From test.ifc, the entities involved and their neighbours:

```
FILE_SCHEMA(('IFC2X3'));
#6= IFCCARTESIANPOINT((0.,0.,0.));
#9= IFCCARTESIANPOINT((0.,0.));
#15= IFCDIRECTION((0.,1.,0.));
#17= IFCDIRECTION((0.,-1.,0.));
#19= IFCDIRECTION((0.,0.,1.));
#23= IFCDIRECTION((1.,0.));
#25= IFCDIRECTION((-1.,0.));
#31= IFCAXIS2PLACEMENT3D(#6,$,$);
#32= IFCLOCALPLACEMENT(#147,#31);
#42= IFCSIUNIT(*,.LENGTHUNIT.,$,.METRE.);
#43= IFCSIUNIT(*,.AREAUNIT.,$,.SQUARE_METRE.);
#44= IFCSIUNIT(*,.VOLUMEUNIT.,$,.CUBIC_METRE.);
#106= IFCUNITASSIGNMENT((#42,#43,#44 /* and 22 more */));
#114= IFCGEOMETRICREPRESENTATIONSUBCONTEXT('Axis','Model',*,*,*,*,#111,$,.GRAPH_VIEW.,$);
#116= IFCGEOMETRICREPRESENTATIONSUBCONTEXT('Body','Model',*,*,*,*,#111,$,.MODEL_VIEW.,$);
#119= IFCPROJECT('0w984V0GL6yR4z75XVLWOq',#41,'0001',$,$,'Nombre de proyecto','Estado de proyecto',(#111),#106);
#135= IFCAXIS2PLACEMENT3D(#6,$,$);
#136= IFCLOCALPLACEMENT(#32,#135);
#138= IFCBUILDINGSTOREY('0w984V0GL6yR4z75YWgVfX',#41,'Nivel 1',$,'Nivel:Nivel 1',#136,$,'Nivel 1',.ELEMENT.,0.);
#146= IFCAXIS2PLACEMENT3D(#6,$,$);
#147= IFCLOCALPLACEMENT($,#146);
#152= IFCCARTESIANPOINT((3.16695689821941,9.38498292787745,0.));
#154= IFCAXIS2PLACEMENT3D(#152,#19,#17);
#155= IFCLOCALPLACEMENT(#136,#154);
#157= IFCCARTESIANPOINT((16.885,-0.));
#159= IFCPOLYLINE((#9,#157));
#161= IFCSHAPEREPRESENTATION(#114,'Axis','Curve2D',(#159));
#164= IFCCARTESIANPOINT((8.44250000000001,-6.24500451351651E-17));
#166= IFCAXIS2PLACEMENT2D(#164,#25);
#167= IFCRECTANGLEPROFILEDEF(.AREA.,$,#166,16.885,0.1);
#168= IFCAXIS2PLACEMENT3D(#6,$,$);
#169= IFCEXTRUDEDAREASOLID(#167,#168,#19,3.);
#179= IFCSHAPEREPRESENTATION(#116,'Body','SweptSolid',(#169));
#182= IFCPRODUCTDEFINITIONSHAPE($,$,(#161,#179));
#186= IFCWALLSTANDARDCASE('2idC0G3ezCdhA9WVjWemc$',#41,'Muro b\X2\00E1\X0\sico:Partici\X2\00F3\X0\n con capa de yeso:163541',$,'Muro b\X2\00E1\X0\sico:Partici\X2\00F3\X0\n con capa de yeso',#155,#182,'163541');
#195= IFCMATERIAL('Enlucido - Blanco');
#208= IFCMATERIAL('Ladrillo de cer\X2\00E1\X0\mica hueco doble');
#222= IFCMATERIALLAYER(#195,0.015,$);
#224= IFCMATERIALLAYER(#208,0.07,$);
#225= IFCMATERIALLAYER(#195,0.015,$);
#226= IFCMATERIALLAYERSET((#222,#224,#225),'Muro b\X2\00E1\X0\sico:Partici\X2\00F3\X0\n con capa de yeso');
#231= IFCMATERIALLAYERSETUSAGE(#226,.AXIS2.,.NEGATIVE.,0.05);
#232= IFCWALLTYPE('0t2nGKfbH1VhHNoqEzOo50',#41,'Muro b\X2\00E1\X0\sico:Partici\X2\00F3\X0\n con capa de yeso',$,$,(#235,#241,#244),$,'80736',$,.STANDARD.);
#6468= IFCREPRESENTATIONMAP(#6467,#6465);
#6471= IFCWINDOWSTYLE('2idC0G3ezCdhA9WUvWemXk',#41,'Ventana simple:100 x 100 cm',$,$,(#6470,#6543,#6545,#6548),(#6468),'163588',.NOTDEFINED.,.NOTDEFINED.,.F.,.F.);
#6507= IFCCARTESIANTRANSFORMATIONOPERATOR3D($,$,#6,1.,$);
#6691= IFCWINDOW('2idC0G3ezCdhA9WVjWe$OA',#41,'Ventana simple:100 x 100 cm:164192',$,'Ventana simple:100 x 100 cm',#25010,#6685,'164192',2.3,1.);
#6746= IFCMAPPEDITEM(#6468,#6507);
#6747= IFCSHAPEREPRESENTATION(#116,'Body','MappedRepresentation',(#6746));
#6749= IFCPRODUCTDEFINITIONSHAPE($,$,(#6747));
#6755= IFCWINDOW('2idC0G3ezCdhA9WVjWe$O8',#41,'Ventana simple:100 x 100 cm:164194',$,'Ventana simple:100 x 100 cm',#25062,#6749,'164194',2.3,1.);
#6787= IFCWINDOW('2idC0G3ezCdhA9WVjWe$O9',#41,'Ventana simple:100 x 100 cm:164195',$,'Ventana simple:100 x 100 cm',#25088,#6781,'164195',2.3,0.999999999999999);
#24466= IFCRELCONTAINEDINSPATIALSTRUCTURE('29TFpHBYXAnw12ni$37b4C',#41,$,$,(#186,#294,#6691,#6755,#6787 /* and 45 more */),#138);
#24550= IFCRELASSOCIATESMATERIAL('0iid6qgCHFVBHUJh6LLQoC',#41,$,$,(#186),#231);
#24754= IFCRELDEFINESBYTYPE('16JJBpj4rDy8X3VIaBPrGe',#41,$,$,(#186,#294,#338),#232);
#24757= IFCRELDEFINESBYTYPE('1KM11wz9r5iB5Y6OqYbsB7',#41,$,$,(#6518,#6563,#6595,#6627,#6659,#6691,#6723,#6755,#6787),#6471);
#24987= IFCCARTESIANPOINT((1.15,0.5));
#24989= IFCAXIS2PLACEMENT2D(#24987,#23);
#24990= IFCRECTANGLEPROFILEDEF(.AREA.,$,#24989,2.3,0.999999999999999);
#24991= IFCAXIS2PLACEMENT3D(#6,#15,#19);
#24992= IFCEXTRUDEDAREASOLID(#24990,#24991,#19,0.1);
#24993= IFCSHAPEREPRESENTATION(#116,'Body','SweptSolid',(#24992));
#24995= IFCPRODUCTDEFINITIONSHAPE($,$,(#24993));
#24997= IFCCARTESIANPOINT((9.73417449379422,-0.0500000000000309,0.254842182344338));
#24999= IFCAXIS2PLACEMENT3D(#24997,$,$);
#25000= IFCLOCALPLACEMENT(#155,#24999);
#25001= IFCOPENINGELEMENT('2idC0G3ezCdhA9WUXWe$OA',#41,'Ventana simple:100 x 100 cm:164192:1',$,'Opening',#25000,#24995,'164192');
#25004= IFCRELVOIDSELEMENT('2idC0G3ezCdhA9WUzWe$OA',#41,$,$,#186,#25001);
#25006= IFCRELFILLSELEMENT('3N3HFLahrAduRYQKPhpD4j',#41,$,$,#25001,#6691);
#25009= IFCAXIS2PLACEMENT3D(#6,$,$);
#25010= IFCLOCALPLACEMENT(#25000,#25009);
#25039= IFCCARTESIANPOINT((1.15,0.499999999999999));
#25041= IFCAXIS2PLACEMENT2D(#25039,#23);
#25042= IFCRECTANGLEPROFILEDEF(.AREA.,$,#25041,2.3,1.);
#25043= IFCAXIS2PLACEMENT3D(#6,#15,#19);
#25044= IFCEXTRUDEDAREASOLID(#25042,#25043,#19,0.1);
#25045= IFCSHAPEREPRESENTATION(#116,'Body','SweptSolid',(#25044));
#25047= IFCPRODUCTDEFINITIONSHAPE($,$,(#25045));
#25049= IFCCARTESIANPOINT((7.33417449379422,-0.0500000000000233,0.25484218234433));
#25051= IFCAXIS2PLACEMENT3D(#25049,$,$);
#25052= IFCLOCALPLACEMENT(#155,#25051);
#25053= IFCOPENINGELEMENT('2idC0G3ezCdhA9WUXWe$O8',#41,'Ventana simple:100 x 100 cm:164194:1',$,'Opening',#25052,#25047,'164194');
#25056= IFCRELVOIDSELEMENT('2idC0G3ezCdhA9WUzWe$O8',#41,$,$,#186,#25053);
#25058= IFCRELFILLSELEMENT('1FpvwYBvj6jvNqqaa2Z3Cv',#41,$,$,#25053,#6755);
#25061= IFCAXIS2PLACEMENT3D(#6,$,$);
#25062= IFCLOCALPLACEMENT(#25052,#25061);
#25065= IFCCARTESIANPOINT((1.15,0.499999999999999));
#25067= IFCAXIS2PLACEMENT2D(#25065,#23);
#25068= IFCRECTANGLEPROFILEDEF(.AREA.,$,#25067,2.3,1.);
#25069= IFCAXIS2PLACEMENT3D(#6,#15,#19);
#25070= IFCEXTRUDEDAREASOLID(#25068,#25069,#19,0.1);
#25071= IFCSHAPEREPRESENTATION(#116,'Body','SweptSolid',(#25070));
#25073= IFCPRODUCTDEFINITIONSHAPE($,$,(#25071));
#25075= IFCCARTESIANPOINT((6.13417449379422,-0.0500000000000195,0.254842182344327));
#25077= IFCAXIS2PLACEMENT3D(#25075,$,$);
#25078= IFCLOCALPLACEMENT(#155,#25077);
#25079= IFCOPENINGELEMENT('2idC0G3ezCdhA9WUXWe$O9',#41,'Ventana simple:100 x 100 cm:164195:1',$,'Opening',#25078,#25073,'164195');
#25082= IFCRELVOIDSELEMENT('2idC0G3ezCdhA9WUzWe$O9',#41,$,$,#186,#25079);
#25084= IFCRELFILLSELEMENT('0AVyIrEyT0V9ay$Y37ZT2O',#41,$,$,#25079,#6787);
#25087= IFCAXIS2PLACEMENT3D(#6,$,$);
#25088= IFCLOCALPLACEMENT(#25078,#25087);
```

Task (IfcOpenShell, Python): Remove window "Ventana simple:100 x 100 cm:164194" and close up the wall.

```python
import ifcopenshell
import ifcopenshell.api.feature
import ifcopenshell.api.root
import ifcopenshell.geom
import ifcopenshell.util.shape

model = ifcopenshell.open("test.ifc")
settings = ifcopenshell.geom.settings()


def volume(element):
    """Net volume in cubic metres, openings subtracted."""
    shape = ifcopenshell.geom.create_shape(settings, element)
    return ifcopenshell.util.shape.get_volume(shape.geometry)


window = model.by_id(6755)
opening = window.FillsVoids[0].RelatingOpeningElement
wall = opening.VoidsElements[0].RelatingBuildingElement
before = volume(wall)

ifcopenshell.api.root.remove_product(model, product=window)
ifcopenshell.api.feature.remove_feature(model, feature=opening)

after = volume(wall)

print(f"wall volume {before:.3f} -> {after:.3f} m3")

model.write("test_rev.ifc")
```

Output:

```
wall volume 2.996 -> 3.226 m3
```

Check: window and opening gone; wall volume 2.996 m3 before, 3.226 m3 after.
